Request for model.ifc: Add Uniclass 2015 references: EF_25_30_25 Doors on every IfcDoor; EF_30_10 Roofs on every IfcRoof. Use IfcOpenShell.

First a look at what the model holds.

```python
import ifcopenshell

model = ifcopenshell.open("model.ifc")
print(model.schema)
print("classifications:", [c.Name for c in model.by_type("IfcClassification")])
for ifc_class in ("IfcDoor", "IfcRoof", "IfcStair", "IfcWall", "IfcWindow"):
    print(ifc_class, len(model.by_type(ifc_class)))
```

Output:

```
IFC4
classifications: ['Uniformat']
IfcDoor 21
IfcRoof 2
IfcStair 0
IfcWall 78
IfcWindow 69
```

```python
import ifcopenshell
import ifcopenshell.api.classification

model = ifcopenshell.open("model.ifc")

system = ifcopenshell.api.classification.add_classification(model, classification="Uniclass 2015")

codes = {
    "IfcDoor": ("EF_25_30_25", "Doors"),
    "IfcRoof": ("EF_30_10", "Roofs"),
}
for ifc_class, (code, name) in codes.items():
    products = model.by_type(ifc_class)
    ifcopenshell.api.classification.add_reference(
        model, products=products, classification=system, identification=code, name=name
    )
    print(code, len(products))

model.write("model_rev.ifc")
```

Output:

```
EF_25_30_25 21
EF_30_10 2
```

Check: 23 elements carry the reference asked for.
